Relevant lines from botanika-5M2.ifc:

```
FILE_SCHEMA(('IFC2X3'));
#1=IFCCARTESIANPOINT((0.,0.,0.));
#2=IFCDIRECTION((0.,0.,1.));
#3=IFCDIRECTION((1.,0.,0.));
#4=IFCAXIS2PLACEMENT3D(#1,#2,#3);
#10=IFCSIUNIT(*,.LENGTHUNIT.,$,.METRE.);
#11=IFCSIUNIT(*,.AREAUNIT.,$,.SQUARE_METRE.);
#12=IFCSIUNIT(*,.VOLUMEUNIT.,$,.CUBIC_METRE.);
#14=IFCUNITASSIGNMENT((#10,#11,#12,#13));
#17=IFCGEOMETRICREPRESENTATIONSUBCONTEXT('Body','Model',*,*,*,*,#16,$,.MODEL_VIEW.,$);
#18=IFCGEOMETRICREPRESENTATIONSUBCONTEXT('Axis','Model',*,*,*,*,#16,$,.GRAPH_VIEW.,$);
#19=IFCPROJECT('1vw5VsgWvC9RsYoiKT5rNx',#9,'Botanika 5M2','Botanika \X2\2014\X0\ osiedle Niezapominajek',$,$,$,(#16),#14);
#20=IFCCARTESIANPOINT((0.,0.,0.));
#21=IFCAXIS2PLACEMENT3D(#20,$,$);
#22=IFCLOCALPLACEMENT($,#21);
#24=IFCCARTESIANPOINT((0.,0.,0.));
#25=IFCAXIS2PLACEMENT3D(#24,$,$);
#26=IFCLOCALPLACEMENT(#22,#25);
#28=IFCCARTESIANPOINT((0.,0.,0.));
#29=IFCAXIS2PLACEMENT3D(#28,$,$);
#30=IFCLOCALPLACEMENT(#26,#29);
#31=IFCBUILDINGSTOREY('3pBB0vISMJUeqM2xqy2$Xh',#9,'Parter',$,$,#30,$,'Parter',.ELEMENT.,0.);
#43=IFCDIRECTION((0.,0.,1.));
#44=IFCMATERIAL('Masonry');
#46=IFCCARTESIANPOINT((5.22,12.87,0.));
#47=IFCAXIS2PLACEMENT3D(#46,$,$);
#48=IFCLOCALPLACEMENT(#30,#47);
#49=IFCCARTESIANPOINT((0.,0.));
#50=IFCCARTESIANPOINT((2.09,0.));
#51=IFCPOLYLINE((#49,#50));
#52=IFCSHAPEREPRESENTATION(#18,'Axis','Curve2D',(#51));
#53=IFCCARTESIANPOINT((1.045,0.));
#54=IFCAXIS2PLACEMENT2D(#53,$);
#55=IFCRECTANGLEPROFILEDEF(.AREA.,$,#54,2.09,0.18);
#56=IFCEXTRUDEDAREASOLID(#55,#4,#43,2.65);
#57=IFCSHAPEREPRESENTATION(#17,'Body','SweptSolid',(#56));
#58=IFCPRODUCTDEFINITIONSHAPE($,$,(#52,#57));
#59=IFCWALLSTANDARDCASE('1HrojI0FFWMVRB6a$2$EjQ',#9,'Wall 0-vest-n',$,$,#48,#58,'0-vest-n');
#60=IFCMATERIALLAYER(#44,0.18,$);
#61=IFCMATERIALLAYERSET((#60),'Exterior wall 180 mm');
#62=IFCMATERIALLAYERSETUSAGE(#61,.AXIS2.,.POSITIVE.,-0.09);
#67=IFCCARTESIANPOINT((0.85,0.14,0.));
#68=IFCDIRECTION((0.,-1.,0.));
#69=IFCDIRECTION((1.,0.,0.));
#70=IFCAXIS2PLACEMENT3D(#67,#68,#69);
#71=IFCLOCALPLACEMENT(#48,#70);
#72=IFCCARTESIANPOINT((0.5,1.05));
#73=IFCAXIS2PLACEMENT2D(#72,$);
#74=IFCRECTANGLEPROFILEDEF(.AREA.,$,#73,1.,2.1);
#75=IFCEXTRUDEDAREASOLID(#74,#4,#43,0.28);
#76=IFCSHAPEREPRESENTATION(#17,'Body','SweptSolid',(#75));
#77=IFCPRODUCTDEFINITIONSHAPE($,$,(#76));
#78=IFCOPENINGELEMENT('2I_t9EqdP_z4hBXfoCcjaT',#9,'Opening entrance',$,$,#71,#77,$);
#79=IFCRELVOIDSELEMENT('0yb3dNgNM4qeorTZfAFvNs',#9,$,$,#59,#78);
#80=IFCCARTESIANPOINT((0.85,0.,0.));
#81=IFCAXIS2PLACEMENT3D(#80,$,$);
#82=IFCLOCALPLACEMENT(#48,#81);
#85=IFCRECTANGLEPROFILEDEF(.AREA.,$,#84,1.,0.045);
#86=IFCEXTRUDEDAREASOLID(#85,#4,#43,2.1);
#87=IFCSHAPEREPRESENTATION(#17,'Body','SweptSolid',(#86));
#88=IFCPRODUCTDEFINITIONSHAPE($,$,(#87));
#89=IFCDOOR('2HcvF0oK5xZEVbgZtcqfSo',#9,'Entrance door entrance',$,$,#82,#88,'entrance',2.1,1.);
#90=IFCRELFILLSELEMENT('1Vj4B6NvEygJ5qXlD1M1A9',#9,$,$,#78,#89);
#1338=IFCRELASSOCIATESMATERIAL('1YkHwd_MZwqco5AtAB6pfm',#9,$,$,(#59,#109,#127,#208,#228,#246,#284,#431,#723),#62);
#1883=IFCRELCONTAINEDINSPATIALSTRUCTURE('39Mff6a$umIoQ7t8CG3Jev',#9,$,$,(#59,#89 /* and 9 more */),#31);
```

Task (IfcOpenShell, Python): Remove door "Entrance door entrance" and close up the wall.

```python
import ifcopenshell
import ifcopenshell.api.feature
import ifcopenshell.api.root
import ifcopenshell.geom
import ifcopenshell.util.shape

model = ifcopenshell.open("botanika-5M2.ifc")
settings = ifcopenshell.geom.settings()


def volume(element):
    """Net volume in cubic metres, openings subtracted."""
    shape = ifcopenshell.geom.create_shape(settings, element)
    return ifcopenshell.util.shape.get_volume(shape.geometry)


door = model.by_guid("2HcvF0oK5xZEVbgZtcqfSo")
opening = door.FillsVoids[0].RelatingOpeningElement
wall = opening.VoidsElements[0].RelatingBuildingElement
before = volume(wall)

ifcopenshell.api.root.remove_product(model, product=door)
ifcopenshell.api.feature.remove_feature(model, feature=opening)

after = volume(wall)

print(f"wall volume {before:.3f} -> {after:.3f} m3")

model.write("botanika-5M2_edited.ifc")
```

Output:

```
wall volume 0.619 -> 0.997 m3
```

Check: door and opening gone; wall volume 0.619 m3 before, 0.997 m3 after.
